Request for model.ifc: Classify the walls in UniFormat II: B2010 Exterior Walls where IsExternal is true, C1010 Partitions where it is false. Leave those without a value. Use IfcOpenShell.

First a look at what the model holds.

```python
import ifcopenshell
import ifcopenshell.util.element

model = ifcopenshell.open("model.ifc")
print(model.schema)
print("classifications:", [c.Name for c in model.by_type("IfcClassification")])
values = [ifcopenshell.util.element.get_pset(e, "Pset_WallCommon", "IsExternal") for e in model.by_type("IfcWall")]
for value in (True, False, None):
    print("IsExternal", value, values.count(value))
```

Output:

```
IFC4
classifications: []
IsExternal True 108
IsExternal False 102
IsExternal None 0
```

```python
import ifcopenshell
import ifcopenshell.api.classification
import ifcopenshell.util.element

model = ifcopenshell.open("model.ifc")

system = ifcopenshell.api.classification.add_classification(model, classification="UniFormat II")

walls = model.by_type("IfcWall")
external = {e: ifcopenshell.util.element.get_pset(e, "Pset_WallCommon", "IsExternal") for e in walls}
for flag, code, name in ((True, "B2010", "Exterior Walls"), (False, "C1010", "Partitions")):
    products = [e for e in walls if external[e] is flag]
    ifcopenshell.api.classification.add_reference(
        model, products=products, classification=system, identification=code, name=name
    )
    print(code, len(products))

model.write("model-out.ifc")
```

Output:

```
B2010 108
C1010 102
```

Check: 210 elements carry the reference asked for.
